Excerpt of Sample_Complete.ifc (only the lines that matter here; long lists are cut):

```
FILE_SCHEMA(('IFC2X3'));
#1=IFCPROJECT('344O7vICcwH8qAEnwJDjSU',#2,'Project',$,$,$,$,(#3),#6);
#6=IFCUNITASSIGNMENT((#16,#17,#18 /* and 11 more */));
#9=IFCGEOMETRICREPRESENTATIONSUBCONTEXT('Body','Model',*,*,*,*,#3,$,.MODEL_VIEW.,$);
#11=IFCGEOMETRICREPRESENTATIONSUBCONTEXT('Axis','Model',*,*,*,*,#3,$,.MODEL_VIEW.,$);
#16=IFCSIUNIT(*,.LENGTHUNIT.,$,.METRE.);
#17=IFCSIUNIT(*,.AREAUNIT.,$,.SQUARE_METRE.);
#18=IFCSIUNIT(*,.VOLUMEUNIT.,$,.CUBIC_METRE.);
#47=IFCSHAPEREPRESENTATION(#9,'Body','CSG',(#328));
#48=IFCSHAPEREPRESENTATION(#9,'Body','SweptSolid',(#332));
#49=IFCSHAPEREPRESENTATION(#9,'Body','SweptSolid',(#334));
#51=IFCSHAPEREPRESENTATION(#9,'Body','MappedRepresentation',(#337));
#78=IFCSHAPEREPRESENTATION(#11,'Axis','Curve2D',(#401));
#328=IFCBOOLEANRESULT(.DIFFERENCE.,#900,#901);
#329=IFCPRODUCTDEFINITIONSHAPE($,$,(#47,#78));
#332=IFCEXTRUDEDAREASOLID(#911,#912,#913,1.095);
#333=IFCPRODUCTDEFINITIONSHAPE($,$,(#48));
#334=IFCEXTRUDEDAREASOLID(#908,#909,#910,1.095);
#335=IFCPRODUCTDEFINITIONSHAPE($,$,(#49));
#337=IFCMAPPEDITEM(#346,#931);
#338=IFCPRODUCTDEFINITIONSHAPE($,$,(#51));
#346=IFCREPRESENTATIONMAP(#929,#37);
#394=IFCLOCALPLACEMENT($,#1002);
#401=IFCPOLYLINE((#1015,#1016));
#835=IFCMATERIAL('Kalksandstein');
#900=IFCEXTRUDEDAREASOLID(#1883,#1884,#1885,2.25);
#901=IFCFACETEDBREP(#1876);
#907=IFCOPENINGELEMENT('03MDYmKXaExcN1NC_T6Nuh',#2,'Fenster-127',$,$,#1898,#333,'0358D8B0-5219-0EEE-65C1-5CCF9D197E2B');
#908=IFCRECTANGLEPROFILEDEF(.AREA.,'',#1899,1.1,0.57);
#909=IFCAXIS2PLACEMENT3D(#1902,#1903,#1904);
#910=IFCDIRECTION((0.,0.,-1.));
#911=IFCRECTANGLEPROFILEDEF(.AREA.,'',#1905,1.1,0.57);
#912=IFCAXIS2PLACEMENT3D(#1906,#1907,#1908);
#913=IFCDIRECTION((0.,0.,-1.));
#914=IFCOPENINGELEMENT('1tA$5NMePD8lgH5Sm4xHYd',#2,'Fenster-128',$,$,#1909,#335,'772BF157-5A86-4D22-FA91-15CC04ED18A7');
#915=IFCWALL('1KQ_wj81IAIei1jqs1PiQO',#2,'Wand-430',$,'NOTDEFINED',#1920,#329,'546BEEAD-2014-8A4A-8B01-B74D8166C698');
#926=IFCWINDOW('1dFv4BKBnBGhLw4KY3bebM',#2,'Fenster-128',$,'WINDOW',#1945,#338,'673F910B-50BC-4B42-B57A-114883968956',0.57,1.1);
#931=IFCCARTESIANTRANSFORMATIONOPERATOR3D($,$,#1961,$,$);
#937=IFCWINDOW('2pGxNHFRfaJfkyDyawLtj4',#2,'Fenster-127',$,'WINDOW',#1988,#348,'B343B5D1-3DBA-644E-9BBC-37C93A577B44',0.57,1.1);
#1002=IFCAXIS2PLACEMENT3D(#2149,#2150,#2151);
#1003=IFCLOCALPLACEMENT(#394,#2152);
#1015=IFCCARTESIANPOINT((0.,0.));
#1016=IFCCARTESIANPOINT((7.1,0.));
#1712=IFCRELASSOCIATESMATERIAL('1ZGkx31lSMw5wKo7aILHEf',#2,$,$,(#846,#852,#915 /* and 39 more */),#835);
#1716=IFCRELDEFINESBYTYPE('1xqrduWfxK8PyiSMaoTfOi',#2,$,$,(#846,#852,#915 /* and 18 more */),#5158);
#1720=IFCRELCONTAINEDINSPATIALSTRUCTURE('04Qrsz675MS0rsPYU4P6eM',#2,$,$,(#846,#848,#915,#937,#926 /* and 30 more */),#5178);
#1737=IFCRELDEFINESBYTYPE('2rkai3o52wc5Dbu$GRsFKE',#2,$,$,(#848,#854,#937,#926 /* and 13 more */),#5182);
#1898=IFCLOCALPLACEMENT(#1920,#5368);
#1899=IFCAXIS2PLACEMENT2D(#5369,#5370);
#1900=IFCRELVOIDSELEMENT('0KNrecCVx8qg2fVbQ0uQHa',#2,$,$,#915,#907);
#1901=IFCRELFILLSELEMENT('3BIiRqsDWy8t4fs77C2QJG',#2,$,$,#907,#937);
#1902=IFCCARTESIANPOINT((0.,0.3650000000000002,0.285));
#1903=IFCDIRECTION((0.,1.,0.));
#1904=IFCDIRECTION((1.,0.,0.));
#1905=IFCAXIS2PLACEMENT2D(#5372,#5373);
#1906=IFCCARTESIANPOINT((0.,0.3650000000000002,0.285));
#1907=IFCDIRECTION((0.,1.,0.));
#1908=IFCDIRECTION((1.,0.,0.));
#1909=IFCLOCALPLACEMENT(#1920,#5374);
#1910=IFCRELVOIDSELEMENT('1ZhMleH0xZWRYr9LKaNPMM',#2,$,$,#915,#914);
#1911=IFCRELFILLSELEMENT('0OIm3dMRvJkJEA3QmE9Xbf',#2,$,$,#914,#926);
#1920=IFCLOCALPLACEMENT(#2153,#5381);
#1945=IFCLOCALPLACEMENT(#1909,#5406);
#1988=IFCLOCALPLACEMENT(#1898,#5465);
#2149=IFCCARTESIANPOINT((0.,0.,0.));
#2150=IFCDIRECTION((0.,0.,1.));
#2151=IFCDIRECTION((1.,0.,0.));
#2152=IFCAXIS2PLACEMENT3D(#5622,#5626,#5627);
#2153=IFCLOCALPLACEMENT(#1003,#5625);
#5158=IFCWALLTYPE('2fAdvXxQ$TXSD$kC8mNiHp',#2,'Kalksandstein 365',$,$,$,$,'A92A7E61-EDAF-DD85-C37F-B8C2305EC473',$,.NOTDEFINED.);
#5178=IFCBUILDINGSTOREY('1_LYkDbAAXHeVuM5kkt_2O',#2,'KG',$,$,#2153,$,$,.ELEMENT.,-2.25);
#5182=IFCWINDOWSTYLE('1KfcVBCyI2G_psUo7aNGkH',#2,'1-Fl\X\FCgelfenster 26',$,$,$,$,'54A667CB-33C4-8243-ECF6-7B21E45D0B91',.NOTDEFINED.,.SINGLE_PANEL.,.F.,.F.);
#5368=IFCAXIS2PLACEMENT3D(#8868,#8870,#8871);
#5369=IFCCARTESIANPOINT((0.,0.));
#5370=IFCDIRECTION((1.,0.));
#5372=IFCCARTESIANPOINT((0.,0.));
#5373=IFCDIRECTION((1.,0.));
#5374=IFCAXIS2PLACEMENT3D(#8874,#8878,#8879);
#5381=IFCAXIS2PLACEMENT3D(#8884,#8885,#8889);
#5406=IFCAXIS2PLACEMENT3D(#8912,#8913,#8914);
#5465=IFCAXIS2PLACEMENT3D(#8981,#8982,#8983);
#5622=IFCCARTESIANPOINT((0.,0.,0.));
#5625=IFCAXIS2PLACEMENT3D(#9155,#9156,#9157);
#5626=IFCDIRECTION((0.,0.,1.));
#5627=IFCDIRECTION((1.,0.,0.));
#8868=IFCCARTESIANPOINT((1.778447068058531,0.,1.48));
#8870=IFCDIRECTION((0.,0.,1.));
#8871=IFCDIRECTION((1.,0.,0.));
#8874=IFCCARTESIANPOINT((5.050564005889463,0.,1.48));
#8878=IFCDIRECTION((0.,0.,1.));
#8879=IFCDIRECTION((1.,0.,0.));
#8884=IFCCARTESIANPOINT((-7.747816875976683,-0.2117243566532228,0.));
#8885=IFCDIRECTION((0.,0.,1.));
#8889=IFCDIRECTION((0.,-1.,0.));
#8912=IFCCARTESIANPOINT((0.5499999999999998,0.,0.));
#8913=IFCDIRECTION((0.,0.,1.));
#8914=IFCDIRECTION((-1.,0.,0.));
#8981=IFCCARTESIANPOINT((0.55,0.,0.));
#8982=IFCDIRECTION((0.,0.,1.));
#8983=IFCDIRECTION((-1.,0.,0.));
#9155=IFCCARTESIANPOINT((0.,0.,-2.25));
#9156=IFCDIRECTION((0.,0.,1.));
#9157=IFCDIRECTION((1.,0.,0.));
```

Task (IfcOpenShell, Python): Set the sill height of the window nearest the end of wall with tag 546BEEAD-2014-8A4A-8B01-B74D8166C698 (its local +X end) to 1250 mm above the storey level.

```python
import numpy as np
import ifcopenshell
import ifcopenshell.api.geometry
import ifcopenshell.geom
import ifcopenshell.util.element
import ifcopenshell.util.placement
import ifcopenshell.util.shape
import ifcopenshell.util.unit

model = ifcopenshell.open("Sample_Complete.ifc")
unit_scale = ifcopenshell.util.unit.calculate_unit_scale(model)

window = model.by_guid("1dFv4BKBnBGhLw4KY3bebM")
opening = window.FillsVoids[0].RelatingOpeningElement
storey = ifcopenshell.util.element.get_container(window, ifc_class="IfcBuildingStorey")
level = ifcopenshell.util.placement.get_local_placement(storey.ObjectPlacement)[2, 3]

# The opening's origin need not be at the sill, so measure its lowest point.
shape = ifcopenshell.geom.create_shape(ifcopenshell.geom.settings(), opening)
bottom = ifcopenshell.util.shape.get_shape_bottom_elevation(shape, shape.geometry) / unit_scale
dz = level + 1.25 - bottom

shift = np.array([0.0, 0.0, dz])
# The window is placed relative to its opening, so it follows when the opening moves.
matrix = ifcopenshell.util.placement.get_local_placement(opening.ObjectPlacement)
matrix[:3, 3] += shift
ifcopenshell.api.geometry.edit_object_placement(
    model, product=opening, matrix=matrix, is_si=False, should_transform_children=True
)

print(f"moved by {dz * unit_scale:+.3f} m")

model.write("Sample_Complete_updated.ifc")
```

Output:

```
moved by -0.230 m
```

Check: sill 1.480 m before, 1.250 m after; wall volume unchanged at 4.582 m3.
